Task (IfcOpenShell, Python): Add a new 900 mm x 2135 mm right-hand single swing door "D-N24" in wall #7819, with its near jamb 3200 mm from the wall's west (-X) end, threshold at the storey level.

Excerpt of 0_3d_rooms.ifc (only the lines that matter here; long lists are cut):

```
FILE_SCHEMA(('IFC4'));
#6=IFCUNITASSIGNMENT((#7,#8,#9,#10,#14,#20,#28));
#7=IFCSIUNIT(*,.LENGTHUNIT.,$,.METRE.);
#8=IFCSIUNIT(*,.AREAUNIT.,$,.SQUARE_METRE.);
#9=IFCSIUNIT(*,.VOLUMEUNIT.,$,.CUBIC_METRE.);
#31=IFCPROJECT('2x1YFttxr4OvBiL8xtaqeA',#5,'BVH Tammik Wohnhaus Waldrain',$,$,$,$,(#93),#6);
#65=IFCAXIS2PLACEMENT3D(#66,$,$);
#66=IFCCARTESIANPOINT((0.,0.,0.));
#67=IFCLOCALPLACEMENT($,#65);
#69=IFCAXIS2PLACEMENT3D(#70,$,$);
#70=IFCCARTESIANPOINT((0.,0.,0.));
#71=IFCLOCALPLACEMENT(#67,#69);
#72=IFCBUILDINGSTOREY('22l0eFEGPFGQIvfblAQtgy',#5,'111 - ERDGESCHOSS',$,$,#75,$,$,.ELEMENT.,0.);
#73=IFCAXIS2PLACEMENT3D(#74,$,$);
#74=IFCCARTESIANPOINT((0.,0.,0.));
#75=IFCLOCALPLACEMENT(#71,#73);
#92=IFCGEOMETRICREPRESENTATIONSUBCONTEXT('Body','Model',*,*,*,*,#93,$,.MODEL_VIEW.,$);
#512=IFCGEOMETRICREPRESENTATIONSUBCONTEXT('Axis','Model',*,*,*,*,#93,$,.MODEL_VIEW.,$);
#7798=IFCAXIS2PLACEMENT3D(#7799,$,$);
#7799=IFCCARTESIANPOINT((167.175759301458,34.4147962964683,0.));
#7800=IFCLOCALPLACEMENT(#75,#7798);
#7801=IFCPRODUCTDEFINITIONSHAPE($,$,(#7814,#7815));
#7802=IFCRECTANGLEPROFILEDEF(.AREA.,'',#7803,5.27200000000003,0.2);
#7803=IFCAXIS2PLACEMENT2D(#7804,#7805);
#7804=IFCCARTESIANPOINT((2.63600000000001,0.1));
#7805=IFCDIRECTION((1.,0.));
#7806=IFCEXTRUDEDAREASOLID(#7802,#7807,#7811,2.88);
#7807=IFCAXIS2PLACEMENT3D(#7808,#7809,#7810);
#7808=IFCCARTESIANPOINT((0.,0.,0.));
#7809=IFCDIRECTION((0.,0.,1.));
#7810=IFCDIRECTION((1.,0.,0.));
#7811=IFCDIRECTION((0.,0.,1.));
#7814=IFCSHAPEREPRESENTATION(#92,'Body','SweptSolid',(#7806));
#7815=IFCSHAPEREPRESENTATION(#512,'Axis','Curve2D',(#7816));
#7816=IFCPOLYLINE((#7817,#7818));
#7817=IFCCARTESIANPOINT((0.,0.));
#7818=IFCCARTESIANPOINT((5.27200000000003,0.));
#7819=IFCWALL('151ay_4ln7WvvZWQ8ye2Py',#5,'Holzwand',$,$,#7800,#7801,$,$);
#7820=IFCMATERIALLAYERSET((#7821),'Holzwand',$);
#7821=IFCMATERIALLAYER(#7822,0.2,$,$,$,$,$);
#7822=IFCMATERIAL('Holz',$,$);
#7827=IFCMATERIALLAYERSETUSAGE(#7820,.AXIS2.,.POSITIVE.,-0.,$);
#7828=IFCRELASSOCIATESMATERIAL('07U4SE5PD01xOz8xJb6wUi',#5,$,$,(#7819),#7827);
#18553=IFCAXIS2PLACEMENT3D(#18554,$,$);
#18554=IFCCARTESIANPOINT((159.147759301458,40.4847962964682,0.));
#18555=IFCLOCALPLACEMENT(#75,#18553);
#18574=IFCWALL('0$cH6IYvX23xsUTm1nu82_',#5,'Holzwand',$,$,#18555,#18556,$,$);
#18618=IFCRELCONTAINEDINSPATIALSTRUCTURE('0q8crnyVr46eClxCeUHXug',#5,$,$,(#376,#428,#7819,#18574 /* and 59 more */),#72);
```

```python
import numpy as np
import ifcopenshell
import ifcopenshell.api.feature
import ifcopenshell.api.geometry
import ifcopenshell.api.root
import ifcopenshell.api.spatial
import ifcopenshell.geom
import ifcopenshell.util.element
import ifcopenshell.util.placement
import ifcopenshell.util.representation
import ifcopenshell.util.shape
import ifcopenshell.util.unit

model = ifcopenshell.open("0_3d_rooms.ifc")
unit_scale = ifcopenshell.util.unit.calculate_unit_scale(model)
settings = ifcopenshell.geom.settings()


def volume(element):
    """Net volume in cubic metres, openings subtracted."""
    shape = ifcopenshell.geom.create_shape(settings, element)
    return ifcopenshell.util.shape.get_volume(shape.geometry)


wall = model.by_id(7819)
storey = ifcopenshell.util.element.get_container(wall, ifc_class="IfcBuildingStorey")
context = ifcopenshell.util.representation.get_context(model, "Model", "Body", "MODEL_VIEW")
before = volume(wall)

width, height, from_end, sill = 0.9, 2.135, 3.2, 0.0  # metres

# The wall runs along its own X axis, and the end named is its -X end.
wall_shape = ifcopenshell.geom.create_shape(settings, wall)
x, y, z = ifcopenshell.util.shape.get_vertices(wall_shape.geometry).T
start = x.min() + from_end
face, thickness = float(y.min()), float(y.max() - y.min())
wall_matrix = ifcopenshell.util.placement.get_local_placement(wall.ObjectPlacement)
level = ifcopenshell.util.placement.get_local_placement(storey.ObjectPlacement)[2, 3]


def in_wall(x, y):
    """Placement at x, y metres in the wall's axes, at sill height."""
    matrix = wall_matrix.copy()
    matrix[:, 3] = wall_matrix @ np.array([x / unit_scale, y / unit_scale, 0.0, 1.0])
    matrix[2, 3] = level + sill / unit_scale
    return matrix


# Opening: a box that overshoots both wall faces by 50 mm.
opening = ifcopenshell.api.root.create_entity(model, ifc_class="IfcOpeningElement", predefined_type="OPENING")
box = ifcopenshell.api.geometry.add_wall_representation(
    model, context=context, length=width, height=height, thickness=thickness + 0.1
)
ifcopenshell.api.geometry.assign_representation(model, product=opening, representation=box)
ifcopenshell.api.geometry.edit_object_placement(model, product=opening, matrix=in_wall(start, face - 0.05), is_si=False)
ifcopenshell.api.feature.add_feature(model, feature=opening, element=wall)

door = ifcopenshell.api.root.create_entity(model, ifc_class="IfcDoor", name="D-N24", predefined_type="DOOR")
door.OverallWidth, door.OverallHeight = width / unit_scale, height / unit_scale
door.OperationType = "SINGLE_SWING_RIGHT"
body = ifcopenshell.api.geometry.add_door_representation(
    model,
    context=context,
    overall_width=door.OverallWidth,
    overall_height=door.OverallHeight,
    operation_type="SINGLE_SWING_RIGHT",
    lining_properties={"LiningDepth": thickness / unit_scale, "ThresholdDepth": thickness / unit_scale},
)
ifcopenshell.api.geometry.assign_representation(model, product=door, representation=body)
ifcopenshell.api.spatial.assign_container(model, products=[door], relating_structure=storey)
ifcopenshell.api.feature.add_filling(model, opening=opening, element=door)

# The lining spans the wall, so the door starts at the wall face.
ifcopenshell.api.geometry.edit_object_placement(model, product=door, matrix=in_wall(start, face), is_si=False)

after = volume(wall)

print(f"wall volume {before:.3f} -> {after:.3f} m3")

model.write("0_3d_rooms_rev.ifc")
```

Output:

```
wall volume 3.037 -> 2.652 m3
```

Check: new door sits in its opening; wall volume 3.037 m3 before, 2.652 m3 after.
